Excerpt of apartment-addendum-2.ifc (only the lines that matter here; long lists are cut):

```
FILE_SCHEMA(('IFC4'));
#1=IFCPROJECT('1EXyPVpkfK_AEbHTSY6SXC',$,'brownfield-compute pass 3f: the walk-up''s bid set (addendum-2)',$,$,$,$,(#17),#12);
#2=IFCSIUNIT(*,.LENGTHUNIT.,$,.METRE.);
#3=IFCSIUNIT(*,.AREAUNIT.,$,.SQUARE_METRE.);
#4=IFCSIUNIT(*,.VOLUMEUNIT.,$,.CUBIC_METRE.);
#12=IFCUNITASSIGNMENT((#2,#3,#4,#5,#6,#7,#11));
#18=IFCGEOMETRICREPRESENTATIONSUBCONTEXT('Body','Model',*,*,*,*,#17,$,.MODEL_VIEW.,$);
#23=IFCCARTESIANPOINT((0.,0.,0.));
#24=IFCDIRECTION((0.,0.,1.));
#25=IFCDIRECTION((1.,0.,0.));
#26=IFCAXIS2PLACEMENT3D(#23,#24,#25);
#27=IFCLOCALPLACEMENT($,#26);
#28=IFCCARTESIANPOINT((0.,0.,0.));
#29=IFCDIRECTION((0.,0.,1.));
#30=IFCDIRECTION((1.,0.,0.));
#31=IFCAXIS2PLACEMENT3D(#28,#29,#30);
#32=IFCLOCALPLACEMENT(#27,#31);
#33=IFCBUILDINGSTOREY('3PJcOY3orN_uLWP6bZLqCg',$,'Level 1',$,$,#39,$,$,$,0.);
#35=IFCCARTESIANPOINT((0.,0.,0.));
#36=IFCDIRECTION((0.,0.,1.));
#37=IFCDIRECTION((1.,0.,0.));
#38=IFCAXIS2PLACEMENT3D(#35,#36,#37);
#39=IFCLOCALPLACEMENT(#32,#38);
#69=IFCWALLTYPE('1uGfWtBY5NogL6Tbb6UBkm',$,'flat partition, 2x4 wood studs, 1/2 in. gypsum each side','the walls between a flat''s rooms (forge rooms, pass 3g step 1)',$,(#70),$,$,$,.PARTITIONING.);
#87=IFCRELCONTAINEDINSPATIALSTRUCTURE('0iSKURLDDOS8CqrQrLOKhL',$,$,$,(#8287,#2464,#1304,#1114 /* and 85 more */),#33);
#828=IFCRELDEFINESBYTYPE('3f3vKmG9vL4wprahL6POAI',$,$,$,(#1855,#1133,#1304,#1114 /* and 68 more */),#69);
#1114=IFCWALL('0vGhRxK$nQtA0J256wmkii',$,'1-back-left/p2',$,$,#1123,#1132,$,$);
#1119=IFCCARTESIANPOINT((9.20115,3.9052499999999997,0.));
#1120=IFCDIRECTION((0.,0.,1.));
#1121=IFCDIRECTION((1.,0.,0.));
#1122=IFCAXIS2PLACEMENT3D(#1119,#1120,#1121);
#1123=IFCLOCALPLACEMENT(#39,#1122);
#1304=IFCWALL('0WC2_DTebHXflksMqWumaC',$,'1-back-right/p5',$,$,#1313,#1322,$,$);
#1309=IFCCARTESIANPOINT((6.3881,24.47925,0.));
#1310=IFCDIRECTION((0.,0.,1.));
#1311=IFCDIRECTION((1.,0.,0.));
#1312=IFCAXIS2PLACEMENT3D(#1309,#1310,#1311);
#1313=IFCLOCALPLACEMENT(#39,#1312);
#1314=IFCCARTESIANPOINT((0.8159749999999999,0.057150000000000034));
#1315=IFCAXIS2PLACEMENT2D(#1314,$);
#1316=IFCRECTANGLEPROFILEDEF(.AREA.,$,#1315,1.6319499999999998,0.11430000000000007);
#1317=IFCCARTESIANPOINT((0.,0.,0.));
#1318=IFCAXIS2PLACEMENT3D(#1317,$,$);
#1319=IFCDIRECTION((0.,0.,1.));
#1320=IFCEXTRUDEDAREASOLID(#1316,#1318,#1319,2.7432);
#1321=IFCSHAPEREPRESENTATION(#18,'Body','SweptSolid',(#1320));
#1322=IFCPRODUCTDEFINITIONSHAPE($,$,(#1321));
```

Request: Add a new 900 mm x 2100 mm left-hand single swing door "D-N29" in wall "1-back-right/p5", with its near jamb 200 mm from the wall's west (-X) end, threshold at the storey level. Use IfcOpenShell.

```python
import numpy as np
import ifcopenshell
import ifcopenshell.api.feature
import ifcopenshell.api.geometry
import ifcopenshell.api.root
import ifcopenshell.api.spatial
import ifcopenshell.geom
import ifcopenshell.util.element
import ifcopenshell.util.placement
import ifcopenshell.util.representation
import ifcopenshell.util.shape
import ifcopenshell.util.unit

model = ifcopenshell.open("apartment-addendum-2.ifc")
unit_scale = ifcopenshell.util.unit.calculate_unit_scale(model)
settings = ifcopenshell.geom.settings()


def volume(element):
    """Net volume in cubic metres, openings subtracted."""
    shape = ifcopenshell.geom.create_shape(settings, element)
    return ifcopenshell.util.shape.get_volume(shape.geometry)


wall = model.by_guid("0WC2_DTebHXflksMqWumaC")
storey = ifcopenshell.util.element.get_container(wall, ifc_class="IfcBuildingStorey")
context = ifcopenshell.util.representation.get_context(model, "Model", "Body", "MODEL_VIEW")
before = volume(wall)

width, height, from_end, sill = 0.9, 2.1, 0.2, 0.0  # metres

# The wall runs along its own X axis, and the end named is its -X end.
wall_shape = ifcopenshell.geom.create_shape(settings, wall)
x, y, z = ifcopenshell.util.shape.get_vertices(wall_shape.geometry).T
start = x.min() + from_end
face, thickness = float(y.min()), float(y.max() - y.min())
wall_matrix = ifcopenshell.util.placement.get_local_placement(wall.ObjectPlacement)
level = ifcopenshell.util.placement.get_local_placement(storey.ObjectPlacement)[2, 3]


def in_wall(x, y):
    """Placement at x, y metres in the wall's axes, at sill height."""
    matrix = wall_matrix.copy()
    matrix[:, 3] = wall_matrix @ np.array([x / unit_scale, y / unit_scale, 0.0, 1.0])
    matrix[2, 3] = level + sill / unit_scale
    return matrix


# Opening: a box that overshoots both wall faces by 50 mm.
opening = ifcopenshell.api.root.create_entity(model, ifc_class="IfcOpeningElement", predefined_type="OPENING")
box = ifcopenshell.api.geometry.add_wall_representation(
    model, context=context, length=width, height=height, thickness=thickness + 0.1
)
ifcopenshell.api.geometry.assign_representation(model, product=opening, representation=box)
ifcopenshell.api.geometry.edit_object_placement(model, product=opening, matrix=in_wall(start, face - 0.05), is_si=False)
ifcopenshell.api.feature.add_feature(model, feature=opening, element=wall)

door = ifcopenshell.api.root.create_entity(model, ifc_class="IfcDoor", name="D-N29", predefined_type="DOOR")
door.OverallWidth, door.OverallHeight = width / unit_scale, height / unit_scale
door.OperationType = "SINGLE_SWING_LEFT"
body = ifcopenshell.api.geometry.add_door_representation(
    model,
    context=context,
    overall_width=door.OverallWidth,
    overall_height=door.OverallHeight,
    operation_type="SINGLE_SWING_LEFT",
    lining_properties={"LiningDepth": thickness / unit_scale, "ThresholdDepth": thickness / unit_scale},
)
ifcopenshell.api.geometry.assign_representation(model, product=door, representation=body)
ifcopenshell.api.spatial.assign_container(model, products=[door], relating_structure=storey)
ifcopenshell.api.feature.add_filling(model, opening=opening, element=door)

# The lining spans the wall, so the door starts at the wall face.
ifcopenshell.api.geometry.edit_object_placement(model, product=door, matrix=in_wall(start, face), is_si=False)

after = volume(wall)

print(f"wall volume {before:.3f} -> {after:.3f} m3")

model.write("apartment-addendum-2_updated.ifc")
```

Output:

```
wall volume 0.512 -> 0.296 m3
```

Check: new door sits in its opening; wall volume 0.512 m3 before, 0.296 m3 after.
